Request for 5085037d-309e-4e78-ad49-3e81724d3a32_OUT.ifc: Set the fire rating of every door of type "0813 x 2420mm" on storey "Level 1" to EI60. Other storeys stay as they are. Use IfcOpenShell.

First a look at what the model holds.

```python
import ifcopenshell
import ifcopenshell.util.element

model = ifcopenshell.open("5085037d-309e-4e78-ad49-3e81724d3a32_OUT.ifc")
print(model.schema)
storey = next(s for s in model.by_type("IfcBuildingStorey") if s.Name == "Level 1")
doors = [e for e in ifcopenshell.util.element.get_decomposition(storey) if e.is_a("IfcDoor")]
seen = {}
for e in doors:
    element_type = ifcopenshell.util.element.get_type(e)
    key = (element_type.Name if element_type != e and element_type else None, ifcopenshell.util.element.get_pset(e, "Pset_DoorCommon", "FireRating"))
    seen[key] = seen.get(key, 0) + 1
for (name, value), count in sorted(seen.items(), key=str):
    print(count, "x", name, "|", value)
```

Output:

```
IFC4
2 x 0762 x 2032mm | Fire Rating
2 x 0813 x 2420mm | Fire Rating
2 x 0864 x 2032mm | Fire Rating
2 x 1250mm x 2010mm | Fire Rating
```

```python
import ifcopenshell
import ifcopenshell.api.pset
import ifcopenshell.util.element

model = ifcopenshell.open("5085037d-309e-4e78-ad49-3e81724d3a32_OUT.ifc")

storey = next(s for s in model.by_type("IfcBuildingStorey") if s.Name == "Level 1")
doors = [e for e in ifcopenshell.util.element.get_decomposition(storey) if e.is_a("IfcDoor")]

count = 0
for e in doors:
    element_type = ifcopenshell.util.element.get_type(e)
    if element_type in (None, e) or element_type.Name != "0813 x 2420mm":
        continue
    # add_pset returns the element's existing set when there is one.
    pset = ifcopenshell.api.pset.add_pset(model, product=e, name="Pset_DoorCommon")
    ifcopenshell.api.pset.edit_pset(model, pset=pset, properties={"FireRating": "EI60"})
    count += 1

print(count, "doors updated")

model.write("5085037d-309e-4e78-ad49-3e81724d3a32_OUT_rev.ifc")
```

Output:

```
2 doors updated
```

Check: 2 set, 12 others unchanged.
